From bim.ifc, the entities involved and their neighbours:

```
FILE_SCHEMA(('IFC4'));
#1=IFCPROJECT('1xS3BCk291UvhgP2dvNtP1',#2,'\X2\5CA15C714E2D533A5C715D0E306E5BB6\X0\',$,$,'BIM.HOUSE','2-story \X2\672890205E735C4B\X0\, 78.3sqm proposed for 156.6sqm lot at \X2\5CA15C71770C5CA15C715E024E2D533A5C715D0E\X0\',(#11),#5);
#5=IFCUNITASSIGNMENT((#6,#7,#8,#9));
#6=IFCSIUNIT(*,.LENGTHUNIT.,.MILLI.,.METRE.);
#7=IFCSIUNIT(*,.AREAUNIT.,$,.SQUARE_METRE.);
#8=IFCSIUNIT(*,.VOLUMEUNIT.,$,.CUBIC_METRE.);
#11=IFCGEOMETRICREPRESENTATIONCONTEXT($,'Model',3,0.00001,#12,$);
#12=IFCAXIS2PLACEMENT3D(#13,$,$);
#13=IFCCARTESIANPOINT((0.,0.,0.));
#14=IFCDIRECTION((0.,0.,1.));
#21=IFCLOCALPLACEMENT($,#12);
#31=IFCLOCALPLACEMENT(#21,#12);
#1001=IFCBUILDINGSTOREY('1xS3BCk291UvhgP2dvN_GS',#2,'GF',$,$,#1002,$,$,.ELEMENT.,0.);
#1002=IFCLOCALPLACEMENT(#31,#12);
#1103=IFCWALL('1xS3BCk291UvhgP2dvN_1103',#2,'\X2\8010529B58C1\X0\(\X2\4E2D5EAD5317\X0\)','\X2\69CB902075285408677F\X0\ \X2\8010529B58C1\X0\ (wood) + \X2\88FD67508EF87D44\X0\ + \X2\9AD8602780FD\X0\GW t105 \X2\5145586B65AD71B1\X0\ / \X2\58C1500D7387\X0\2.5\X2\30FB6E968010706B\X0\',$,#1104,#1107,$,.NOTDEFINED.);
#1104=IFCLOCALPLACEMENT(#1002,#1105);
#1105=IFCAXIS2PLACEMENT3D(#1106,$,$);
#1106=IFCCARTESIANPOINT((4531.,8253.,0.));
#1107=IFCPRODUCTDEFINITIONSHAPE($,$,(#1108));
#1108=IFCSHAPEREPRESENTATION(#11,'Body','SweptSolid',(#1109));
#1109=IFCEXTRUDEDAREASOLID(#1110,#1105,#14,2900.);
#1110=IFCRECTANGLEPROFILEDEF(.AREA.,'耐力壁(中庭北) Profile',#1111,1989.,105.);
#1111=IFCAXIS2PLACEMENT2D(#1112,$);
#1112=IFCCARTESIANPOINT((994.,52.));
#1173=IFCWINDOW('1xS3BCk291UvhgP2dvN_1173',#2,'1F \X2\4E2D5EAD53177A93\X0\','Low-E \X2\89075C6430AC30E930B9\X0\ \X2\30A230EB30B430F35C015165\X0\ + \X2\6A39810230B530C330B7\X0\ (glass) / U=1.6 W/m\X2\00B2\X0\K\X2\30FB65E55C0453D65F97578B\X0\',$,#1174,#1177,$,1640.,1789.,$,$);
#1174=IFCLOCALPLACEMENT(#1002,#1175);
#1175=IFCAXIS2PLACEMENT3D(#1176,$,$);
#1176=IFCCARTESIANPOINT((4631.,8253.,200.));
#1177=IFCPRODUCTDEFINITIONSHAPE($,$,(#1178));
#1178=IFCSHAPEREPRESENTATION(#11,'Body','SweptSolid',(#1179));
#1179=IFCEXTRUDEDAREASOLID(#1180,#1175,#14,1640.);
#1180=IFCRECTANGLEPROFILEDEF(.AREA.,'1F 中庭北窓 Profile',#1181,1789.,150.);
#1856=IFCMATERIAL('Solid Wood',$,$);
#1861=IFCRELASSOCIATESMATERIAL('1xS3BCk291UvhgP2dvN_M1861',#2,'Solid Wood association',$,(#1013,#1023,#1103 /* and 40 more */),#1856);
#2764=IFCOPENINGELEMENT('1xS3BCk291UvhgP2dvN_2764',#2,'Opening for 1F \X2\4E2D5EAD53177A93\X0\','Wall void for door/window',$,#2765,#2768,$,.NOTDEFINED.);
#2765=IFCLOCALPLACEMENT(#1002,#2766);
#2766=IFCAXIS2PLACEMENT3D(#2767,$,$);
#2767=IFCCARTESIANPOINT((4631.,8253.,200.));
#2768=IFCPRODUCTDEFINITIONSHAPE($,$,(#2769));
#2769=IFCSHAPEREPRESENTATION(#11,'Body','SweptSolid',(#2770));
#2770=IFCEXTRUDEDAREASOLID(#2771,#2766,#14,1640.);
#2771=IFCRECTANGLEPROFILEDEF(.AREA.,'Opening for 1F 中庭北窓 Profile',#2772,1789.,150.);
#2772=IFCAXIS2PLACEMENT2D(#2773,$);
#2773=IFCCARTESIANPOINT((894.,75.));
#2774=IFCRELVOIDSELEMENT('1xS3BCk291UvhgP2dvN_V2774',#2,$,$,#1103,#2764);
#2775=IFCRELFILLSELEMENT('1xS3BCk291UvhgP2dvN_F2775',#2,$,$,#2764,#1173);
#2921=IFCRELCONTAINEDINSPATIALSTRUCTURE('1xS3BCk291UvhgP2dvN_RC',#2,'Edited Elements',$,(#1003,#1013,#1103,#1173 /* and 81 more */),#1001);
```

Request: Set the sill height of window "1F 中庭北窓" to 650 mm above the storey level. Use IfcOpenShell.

```python
import numpy as np
import ifcopenshell
import ifcopenshell.api.geometry
import ifcopenshell.geom
import ifcopenshell.util.element
import ifcopenshell.util.placement
import ifcopenshell.util.shape
import ifcopenshell.util.unit

model = ifcopenshell.open("bim.ifc")
unit_scale = ifcopenshell.util.unit.calculate_unit_scale(model)

window = model.by_guid("1xS3BCk291UvhgP2dvN_1173")
opening = window.FillsVoids[0].RelatingOpeningElement
storey = ifcopenshell.util.element.get_container(window, ifc_class="IfcBuildingStorey")
level = ifcopenshell.util.placement.get_local_placement(storey.ObjectPlacement)[2, 3]

# The opening's origin need not be at the sill, so measure its lowest point.
shape = ifcopenshell.geom.create_shape(ifcopenshell.geom.settings(), opening)
bottom = ifcopenshell.util.shape.get_shape_bottom_elevation(shape, shape.geometry) / unit_scale
dz = level + 0.65 / unit_scale - bottom

shift = np.array([0.0, 0.0, dz])
# The window is not placed relative to its opening, so move both.
for product in (opening, window):
    matrix = ifcopenshell.util.placement.get_local_placement(product.ObjectPlacement)
    matrix[:3, 3] += shift
    ifcopenshell.api.geometry.edit_object_placement(model, product=product, matrix=matrix, is_si=False)

print(f"moved by {dz * unit_scale:+.3f} m")

model.write("bim_edited.ifc")
```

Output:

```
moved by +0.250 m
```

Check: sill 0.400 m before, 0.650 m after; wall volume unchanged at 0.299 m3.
